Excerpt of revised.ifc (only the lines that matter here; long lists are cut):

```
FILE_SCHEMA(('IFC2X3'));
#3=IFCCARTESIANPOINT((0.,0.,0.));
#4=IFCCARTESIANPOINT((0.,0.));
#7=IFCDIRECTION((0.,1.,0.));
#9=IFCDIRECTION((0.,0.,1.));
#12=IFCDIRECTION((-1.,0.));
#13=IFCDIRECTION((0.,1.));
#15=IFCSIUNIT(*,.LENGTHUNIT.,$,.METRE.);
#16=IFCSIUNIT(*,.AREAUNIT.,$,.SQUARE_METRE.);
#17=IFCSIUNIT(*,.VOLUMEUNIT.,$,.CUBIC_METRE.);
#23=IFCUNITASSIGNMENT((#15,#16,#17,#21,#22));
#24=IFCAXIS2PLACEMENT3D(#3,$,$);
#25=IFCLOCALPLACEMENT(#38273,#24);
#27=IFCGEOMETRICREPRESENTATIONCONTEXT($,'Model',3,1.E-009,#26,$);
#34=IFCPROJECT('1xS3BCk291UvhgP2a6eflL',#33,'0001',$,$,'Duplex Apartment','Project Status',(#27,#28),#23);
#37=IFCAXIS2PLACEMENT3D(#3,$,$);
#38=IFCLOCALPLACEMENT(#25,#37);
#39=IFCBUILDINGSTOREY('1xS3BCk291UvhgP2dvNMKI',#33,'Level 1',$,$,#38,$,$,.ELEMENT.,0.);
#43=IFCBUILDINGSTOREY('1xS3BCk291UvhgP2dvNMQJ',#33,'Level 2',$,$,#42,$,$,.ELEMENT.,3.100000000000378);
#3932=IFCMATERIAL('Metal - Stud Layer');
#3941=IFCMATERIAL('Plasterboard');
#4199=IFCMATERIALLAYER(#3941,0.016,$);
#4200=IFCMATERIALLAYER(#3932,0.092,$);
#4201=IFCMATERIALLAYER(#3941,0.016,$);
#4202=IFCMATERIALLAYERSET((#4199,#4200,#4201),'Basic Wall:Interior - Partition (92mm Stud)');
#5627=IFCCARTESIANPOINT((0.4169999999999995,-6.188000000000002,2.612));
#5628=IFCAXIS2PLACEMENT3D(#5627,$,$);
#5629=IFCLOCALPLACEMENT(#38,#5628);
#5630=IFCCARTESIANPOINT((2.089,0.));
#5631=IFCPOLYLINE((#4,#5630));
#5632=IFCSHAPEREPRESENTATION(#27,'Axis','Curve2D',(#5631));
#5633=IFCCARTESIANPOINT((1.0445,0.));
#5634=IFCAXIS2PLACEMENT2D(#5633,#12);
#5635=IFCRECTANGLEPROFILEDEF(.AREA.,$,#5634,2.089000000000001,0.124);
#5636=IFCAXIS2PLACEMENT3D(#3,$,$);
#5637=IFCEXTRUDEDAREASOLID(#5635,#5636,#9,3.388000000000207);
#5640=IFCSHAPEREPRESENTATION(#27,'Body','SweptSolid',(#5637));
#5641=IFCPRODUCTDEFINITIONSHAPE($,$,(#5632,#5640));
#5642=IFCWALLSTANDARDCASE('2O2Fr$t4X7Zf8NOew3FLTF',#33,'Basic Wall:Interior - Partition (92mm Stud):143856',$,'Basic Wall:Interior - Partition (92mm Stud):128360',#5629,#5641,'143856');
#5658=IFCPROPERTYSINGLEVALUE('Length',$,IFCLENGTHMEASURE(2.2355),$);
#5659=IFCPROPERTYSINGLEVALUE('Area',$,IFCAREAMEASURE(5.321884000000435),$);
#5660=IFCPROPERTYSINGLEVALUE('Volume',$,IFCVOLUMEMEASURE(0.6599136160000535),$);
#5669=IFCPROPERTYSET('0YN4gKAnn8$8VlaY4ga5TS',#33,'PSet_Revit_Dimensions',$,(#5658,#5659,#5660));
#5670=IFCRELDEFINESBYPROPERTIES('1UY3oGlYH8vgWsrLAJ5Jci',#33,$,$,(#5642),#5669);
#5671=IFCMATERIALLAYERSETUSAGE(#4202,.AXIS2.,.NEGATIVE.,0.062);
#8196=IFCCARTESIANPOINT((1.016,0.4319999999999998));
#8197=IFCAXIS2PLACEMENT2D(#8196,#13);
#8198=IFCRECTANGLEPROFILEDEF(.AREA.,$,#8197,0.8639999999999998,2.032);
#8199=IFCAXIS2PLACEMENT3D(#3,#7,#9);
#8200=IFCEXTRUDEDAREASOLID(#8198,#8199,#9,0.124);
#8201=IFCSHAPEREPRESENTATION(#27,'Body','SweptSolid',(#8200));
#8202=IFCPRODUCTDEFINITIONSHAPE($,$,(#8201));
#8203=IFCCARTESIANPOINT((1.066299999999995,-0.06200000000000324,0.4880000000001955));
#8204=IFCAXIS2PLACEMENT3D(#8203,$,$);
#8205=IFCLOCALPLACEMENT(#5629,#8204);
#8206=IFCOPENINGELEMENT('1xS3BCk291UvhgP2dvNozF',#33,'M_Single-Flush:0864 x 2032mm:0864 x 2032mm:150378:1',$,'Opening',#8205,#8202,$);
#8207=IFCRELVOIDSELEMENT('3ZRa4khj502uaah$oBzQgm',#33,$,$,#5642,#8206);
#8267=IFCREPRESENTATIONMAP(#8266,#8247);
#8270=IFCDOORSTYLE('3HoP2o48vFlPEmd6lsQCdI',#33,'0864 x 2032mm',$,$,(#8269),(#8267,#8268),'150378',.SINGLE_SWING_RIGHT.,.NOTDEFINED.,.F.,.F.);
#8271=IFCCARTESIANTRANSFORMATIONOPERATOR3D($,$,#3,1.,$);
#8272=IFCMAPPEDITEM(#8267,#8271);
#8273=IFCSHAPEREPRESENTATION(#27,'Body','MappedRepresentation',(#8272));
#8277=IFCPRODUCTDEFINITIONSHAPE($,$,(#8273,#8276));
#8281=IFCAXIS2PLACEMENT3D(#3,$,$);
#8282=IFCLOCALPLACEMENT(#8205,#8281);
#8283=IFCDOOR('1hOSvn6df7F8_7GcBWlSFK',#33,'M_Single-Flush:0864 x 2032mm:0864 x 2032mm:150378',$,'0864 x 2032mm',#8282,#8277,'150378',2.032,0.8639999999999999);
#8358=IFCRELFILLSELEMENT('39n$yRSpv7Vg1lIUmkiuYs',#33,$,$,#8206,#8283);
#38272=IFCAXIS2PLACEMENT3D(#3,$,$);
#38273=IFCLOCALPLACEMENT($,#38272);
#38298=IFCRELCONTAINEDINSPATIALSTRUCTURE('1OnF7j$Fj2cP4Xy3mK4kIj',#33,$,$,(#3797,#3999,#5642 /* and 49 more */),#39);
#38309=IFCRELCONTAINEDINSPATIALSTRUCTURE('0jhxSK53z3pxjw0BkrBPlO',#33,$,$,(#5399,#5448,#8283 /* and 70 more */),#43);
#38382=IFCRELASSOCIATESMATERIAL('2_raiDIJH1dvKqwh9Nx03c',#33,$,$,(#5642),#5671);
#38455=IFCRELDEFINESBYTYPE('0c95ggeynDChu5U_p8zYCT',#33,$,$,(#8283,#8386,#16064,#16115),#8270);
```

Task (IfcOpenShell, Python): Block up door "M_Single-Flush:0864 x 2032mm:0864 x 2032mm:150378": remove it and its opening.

```python
import ifcopenshell
import ifcopenshell.api.feature
import ifcopenshell.api.pset
import ifcopenshell.api.root
import ifcopenshell.geom
import ifcopenshell.util.element
import ifcopenshell.util.shape
import ifcopenshell.util.unit

model = ifcopenshell.open("revised.ifc")
area_scale = ifcopenshell.util.unit.calculate_unit_scale(model, "AREAUNIT")
volume_scale = ifcopenshell.util.unit.calculate_unit_scale(model, "VOLUMEUNIT")
settings = ifcopenshell.geom.settings()


def volume(element):
    """Net volume in cubic metres, openings subtracted."""
    shape = ifcopenshell.geom.create_shape(settings, element)
    return ifcopenshell.util.shape.get_volume(shape.geometry)


door = model.by_id(8283)
opening = door.FillsVoids[0].RelatingOpeningElement
wall = opening.VoidsElements[0].RelatingBuildingElement
before = volume(wall)

ifcopenshell.api.root.remove_product(model, product=door)
ifcopenshell.api.feature.remove_feature(model, feature=opening)

after = volume(wall)
thickness = 0.124  # wall thickness in metres

# Update the wall's stored quantities.
pset = model.by_id(ifcopenshell.util.element.get_pset(wall, "PSet_Revit_Dimensions", should_inherit=False)["id"])
ifcopenshell.api.pset.edit_pset(model, pset=pset, properties={
    "Area": model.create_entity("IfcAreaMeasure", after / thickness / area_scale),
    "Volume": model.create_entity("IfcVolumeMeasure", after / volume_scale),
})

print(f"wall volume {before:.3f} -> {after:.3f} m3")

model.write("revised_rev.ifc")
```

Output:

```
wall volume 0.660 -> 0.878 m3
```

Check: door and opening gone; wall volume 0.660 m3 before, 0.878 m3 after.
